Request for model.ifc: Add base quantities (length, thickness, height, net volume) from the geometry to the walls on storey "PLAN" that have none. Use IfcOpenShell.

First a look at what the model holds.

```python
import ifcopenshell
import ifcopenshell.util.element
import ifcopenshell.util.unit

model = ifcopenshell.open("model.ifc")
print(model.schema)
for unit_type in ("LENGTHUNIT", "AREAUNIT", "VOLUMEUNIT"):
    print(unit_type, ifcopenshell.util.unit.calculate_unit_scale(model, unit_type))
storey = next(s for s in model.by_type("IfcBuildingStorey") if s.Name == "PLAN")
walls = [e for e in ifcopenshell.util.element.get_decomposition(storey) if e.is_a("IfcWall")]
for e in sorted(walls, key=lambda e: e.id()):
    print(e.id(), e.is_a(), e.Name, list(ifcopenshell.util.element.get_psets(e, qtos_only=True)), sep=" | ")
```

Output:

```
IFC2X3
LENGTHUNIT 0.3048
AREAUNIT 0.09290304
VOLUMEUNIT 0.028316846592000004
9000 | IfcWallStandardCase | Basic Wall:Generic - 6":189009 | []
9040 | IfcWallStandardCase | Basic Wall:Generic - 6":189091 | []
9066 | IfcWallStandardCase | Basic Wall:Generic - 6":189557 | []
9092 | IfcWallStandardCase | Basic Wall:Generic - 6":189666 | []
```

```python
import ifcopenshell
import ifcopenshell.api.pset
import ifcopenshell.geom
import ifcopenshell.util.element
import ifcopenshell.util.shape
import ifcopenshell.util.unit

model = ifcopenshell.open("model.ifc")
unit_scale = ifcopenshell.util.unit.calculate_unit_scale(model)
volume_scale = ifcopenshell.util.unit.calculate_unit_scale(model, "VOLUMEUNIT")
settings = ifcopenshell.geom.settings()

storey = next(s for s in model.by_type("IfcBuildingStorey") if s.Name == "PLAN")
walls = [e for e in ifcopenshell.util.element.get_decomposition(storey) if e.is_a("IfcWall")]

for e in sorted(walls, key=lambda e: e.id()):
    if ifcopenshell.util.element.get_psets(e, qtos_only=True, should_inherit=False):
        continue
    # Geometry comes back in metres, in the element's own axes.
    shape = ifcopenshell.geom.create_shape(settings, e)
    values = {
        "Length": ifcopenshell.util.shape.get_x(shape.geometry) / unit_scale,
        "Width": ifcopenshell.util.shape.get_y(shape.geometry) / unit_scale,
        "Height": ifcopenshell.util.shape.get_z(shape.geometry) / unit_scale,
        "NetVolume": ifcopenshell.util.shape.get_volume(shape.geometry) / volume_scale,
    }
    qto = ifcopenshell.api.pset.add_qto(model, product=e, name="BaseQuantities")
    ifcopenshell.api.pset.edit_qto(model, qto=qto, properties=values)
    print(e.id(), {k: round(v, 3) for k, v in values.items()})

model.write("model-out.ifc")
```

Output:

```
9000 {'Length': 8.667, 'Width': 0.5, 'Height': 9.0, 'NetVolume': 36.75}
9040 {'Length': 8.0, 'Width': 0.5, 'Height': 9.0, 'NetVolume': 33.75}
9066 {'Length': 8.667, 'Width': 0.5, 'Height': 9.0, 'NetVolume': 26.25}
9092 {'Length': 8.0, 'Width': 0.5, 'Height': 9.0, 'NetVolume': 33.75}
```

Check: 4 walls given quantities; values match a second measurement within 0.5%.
